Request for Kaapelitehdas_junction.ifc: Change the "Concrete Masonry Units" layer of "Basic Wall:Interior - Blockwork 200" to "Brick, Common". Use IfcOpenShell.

First a look at what the model holds.

```python
import ifcopenshell
import ifcopenshell.util.element

model = ifcopenshell.open("Kaapelitehdas_junction.ifc")
print(model.schema)
for layer_set in model.by_type("IfcMaterialLayerSet"):
    if layer_set.LayerSetName == "Basic Wall:Interior - Blockwork 200":
        for layer in layer_set.MaterialLayers:
            print(layer.id(), layer.Material and layer.Material.Name, layer.LayerThickness, sep=" | ")
        print(len(ifcopenshell.util.element.get_elements_by_material(model, layer_set)), "elements and types use it")
print(sorted(m.Name for m in model.by_type("IfcMaterial") if m.Name)[:60])
```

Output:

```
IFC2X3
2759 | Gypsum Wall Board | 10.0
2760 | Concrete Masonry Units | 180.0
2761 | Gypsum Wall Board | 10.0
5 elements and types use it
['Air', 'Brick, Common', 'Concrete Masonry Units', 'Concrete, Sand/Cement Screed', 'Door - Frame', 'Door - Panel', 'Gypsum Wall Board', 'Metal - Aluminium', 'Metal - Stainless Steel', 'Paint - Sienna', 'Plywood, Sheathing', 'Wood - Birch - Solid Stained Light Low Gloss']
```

```python
import ifcopenshell
import ifcopenshell.api.material

model = ifcopenshell.open("Kaapelitehdas_junction.ifc")

layer_set = next(s for s in model.by_type("IfcMaterialLayerSet") if s.LayerSetName == "Basic Wall:Interior - Blockwork 200")
layer = next(l for l in layer_set.MaterialLayers if l.Material and l.Material.Name == "Concrete Masonry Units")
material = next(m for m in model.by_type("IfcMaterial") if m.Name == "Brick, Common")

# Point this one layer at the other material; renaming the old one would change it everywhere.
ifcopenshell.api.material.edit_layer(model, layer=layer, attributes={}, material=material)

print([l.Material.Name if l.Material else None for l in layer_set.MaterialLayers])

model.write("Kaapelitehdas_junction_edited.ifc")
```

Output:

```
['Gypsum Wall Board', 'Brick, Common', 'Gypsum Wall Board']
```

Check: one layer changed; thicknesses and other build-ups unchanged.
